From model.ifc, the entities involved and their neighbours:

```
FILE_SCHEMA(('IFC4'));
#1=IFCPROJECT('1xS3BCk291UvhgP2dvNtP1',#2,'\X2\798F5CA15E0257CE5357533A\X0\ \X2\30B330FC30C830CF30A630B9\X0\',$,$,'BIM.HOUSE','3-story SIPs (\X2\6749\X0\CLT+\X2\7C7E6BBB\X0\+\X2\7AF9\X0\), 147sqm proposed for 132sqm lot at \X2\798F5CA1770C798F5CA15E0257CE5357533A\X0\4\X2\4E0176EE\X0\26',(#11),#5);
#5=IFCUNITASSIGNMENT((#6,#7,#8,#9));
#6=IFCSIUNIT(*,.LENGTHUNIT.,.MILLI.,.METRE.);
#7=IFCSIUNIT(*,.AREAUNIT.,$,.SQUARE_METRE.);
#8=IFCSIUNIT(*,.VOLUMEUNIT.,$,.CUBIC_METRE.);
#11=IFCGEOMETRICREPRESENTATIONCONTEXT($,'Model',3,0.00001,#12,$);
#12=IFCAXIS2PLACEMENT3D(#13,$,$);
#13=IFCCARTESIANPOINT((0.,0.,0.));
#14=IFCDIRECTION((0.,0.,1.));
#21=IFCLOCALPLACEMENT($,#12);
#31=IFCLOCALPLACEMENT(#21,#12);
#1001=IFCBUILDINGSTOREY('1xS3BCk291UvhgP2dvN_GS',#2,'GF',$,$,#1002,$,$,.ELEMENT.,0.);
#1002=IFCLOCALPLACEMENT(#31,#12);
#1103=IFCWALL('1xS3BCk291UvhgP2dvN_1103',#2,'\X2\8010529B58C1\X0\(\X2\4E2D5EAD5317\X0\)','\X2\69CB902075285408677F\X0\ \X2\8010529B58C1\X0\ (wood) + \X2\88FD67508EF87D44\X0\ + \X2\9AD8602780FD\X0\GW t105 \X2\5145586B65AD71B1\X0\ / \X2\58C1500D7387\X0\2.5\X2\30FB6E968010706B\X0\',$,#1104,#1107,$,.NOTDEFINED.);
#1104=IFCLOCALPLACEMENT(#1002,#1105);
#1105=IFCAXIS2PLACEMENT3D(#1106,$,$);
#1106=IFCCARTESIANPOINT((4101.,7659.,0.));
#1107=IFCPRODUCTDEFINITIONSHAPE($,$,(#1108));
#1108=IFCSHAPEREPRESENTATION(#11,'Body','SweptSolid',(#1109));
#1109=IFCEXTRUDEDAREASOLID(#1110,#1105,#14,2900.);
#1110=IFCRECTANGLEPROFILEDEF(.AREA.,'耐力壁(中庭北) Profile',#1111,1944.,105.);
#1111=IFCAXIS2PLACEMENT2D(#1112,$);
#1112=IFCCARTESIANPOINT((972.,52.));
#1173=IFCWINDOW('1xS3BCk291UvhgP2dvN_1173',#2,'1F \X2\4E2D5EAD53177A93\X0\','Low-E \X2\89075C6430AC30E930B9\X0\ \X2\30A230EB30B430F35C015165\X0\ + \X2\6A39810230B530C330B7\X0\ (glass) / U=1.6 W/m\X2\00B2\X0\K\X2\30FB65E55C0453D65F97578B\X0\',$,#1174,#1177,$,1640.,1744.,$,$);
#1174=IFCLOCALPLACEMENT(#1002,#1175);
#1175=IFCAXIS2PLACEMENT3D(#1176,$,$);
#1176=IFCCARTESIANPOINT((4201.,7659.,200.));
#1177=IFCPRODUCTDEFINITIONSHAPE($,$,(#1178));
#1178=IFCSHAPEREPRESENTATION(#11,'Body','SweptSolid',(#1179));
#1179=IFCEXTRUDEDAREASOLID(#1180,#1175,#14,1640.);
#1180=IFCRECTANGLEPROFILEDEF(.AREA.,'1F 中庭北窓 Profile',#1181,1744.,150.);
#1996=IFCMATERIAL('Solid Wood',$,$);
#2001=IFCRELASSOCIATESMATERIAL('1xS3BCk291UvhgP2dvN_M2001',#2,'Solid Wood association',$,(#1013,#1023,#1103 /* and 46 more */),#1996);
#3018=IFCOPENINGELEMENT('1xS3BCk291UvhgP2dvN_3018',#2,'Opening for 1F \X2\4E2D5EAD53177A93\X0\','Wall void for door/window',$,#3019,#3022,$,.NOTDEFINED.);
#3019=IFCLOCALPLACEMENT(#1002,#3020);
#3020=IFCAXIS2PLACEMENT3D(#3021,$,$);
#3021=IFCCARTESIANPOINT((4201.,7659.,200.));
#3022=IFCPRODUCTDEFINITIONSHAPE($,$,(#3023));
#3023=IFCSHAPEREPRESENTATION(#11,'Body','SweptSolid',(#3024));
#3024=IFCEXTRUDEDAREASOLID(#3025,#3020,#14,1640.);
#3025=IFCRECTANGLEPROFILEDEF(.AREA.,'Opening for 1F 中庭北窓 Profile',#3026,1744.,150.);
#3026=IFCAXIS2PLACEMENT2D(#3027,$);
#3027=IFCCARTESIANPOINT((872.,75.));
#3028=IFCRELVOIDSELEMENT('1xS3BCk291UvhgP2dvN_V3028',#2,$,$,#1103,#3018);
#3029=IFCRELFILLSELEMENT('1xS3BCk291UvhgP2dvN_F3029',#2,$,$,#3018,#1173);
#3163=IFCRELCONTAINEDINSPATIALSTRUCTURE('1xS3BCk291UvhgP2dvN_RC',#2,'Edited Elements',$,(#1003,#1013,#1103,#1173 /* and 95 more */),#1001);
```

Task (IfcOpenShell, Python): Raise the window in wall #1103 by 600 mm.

```python
import numpy as np
import ifcopenshell
import ifcopenshell.api.geometry
import ifcopenshell.util.placement
import ifcopenshell.util.unit

model = ifcopenshell.open("model.ifc")
unit_scale = ifcopenshell.util.unit.calculate_unit_scale(model)

window = model.by_id(1173)
opening = window.FillsVoids[0].RelatingOpeningElement
dz = 0.6 / unit_scale

shift = np.array([0.0, 0.0, dz])
# The window is not placed relative to its opening, so move both.
for product in (opening, window):
    matrix = ifcopenshell.util.placement.get_local_placement(product.ObjectPlacement)
    matrix[:3, 3] += shift
    ifcopenshell.api.geometry.edit_object_placement(model, product=product, matrix=matrix, is_si=False)

print(f"moved by {dz * unit_scale:+.3f} m")

model.write("model-out.ifc")
```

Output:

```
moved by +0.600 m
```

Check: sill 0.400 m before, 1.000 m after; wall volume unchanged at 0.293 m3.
